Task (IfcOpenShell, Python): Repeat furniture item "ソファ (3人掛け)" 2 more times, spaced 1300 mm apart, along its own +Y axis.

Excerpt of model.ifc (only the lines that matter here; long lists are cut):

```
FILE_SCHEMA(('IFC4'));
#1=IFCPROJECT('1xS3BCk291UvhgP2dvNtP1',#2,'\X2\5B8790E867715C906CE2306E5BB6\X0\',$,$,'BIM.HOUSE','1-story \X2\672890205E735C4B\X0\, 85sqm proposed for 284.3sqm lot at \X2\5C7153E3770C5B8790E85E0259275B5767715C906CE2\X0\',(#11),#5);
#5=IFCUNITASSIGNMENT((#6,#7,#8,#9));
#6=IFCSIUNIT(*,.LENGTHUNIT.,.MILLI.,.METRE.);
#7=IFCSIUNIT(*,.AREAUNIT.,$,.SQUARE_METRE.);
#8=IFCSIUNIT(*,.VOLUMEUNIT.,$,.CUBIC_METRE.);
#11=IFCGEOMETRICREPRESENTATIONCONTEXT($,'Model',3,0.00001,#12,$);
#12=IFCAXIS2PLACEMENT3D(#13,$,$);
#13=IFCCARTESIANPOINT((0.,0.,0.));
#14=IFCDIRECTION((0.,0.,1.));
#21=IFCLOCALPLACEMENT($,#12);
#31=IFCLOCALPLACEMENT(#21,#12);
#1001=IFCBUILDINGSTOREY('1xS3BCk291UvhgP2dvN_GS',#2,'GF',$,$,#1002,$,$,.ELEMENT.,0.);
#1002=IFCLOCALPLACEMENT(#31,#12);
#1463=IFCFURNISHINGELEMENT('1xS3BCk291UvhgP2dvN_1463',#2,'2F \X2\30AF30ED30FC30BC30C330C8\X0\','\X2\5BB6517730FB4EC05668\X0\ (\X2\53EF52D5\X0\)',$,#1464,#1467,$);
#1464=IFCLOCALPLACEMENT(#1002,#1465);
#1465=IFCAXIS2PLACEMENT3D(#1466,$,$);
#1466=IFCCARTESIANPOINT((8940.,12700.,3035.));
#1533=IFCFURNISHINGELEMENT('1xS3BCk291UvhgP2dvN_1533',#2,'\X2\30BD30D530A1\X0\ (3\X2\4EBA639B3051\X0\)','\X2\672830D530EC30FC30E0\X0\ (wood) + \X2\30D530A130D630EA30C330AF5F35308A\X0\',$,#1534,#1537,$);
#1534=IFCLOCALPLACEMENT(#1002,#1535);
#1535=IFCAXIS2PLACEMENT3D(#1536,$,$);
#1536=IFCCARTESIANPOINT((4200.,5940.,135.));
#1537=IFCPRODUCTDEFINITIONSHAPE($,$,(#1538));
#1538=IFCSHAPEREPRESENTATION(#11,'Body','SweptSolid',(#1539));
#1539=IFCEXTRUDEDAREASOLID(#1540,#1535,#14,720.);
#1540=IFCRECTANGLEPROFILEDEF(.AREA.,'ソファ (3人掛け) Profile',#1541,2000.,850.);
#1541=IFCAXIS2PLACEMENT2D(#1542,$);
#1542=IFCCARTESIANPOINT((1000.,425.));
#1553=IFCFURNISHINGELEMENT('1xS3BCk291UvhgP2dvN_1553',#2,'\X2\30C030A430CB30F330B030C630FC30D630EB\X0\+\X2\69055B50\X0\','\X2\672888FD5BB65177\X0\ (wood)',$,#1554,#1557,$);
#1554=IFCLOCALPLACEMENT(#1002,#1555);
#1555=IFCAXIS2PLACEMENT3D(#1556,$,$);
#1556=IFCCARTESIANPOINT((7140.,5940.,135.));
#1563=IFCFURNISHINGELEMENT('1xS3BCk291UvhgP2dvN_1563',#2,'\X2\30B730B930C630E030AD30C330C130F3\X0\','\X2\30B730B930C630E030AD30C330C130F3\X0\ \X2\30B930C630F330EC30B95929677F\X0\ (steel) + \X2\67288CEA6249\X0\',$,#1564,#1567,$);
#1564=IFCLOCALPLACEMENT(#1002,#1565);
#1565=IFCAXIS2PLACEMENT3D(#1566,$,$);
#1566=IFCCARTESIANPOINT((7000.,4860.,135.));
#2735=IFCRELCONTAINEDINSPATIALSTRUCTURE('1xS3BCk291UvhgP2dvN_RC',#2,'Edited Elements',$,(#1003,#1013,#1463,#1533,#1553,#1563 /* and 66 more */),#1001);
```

```python
import ifcopenshell
import ifcopenshell.api.geometry
import ifcopenshell.api.root
import ifcopenshell.util.element
import ifcopenshell.util.placement
import ifcopenshell.util.unit

model = ifcopenshell.open("model.ifc")
unit_scale = ifcopenshell.util.unit.calculate_unit_scale(model)


def reuse_history(source, copy):
    """copy_class also copies each property set's owner history, people and application; keep the originals."""
    for rel in copy.IsDefinedBy:
        if rel.is_a("IfcRelDefinesByProperties") and (history := rel.RelatingPropertyDefinition.OwnerHistory):
            rel.RelatingPropertyDefinition.OwnerHistory = source.OwnerHistory
            ifcopenshell.util.element.remove_deep2(model, history)


source = model.by_guid("1xS3BCk291UvhgP2dvN_1533")
base = ifcopenshell.util.placement.get_local_placement(source.ObjectPlacement)
step = base[:3, 1] * 1.3 / unit_scale

for i in range(1, 3):
    copy = ifcopenshell.api.root.copy_class(model, product=source)
    copy.Representation = ifcopenshell.util.element.copy_deep(
        model, source.Representation, exclude=["IfcGeometricRepresentationContext", "IfcRepresentationMap"]
    )
    reuse_history(source, copy)
    matrix = base.copy()
    matrix[:3, 3] += i * step
    print("added at", matrix[:3, 3].round(3) + 0.0)
    ifcopenshell.api.geometry.edit_object_placement(model, product=copy, matrix=matrix, is_si=False)

model.write("model_edited.ifc")
```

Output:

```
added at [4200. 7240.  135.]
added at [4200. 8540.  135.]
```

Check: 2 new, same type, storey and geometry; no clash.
